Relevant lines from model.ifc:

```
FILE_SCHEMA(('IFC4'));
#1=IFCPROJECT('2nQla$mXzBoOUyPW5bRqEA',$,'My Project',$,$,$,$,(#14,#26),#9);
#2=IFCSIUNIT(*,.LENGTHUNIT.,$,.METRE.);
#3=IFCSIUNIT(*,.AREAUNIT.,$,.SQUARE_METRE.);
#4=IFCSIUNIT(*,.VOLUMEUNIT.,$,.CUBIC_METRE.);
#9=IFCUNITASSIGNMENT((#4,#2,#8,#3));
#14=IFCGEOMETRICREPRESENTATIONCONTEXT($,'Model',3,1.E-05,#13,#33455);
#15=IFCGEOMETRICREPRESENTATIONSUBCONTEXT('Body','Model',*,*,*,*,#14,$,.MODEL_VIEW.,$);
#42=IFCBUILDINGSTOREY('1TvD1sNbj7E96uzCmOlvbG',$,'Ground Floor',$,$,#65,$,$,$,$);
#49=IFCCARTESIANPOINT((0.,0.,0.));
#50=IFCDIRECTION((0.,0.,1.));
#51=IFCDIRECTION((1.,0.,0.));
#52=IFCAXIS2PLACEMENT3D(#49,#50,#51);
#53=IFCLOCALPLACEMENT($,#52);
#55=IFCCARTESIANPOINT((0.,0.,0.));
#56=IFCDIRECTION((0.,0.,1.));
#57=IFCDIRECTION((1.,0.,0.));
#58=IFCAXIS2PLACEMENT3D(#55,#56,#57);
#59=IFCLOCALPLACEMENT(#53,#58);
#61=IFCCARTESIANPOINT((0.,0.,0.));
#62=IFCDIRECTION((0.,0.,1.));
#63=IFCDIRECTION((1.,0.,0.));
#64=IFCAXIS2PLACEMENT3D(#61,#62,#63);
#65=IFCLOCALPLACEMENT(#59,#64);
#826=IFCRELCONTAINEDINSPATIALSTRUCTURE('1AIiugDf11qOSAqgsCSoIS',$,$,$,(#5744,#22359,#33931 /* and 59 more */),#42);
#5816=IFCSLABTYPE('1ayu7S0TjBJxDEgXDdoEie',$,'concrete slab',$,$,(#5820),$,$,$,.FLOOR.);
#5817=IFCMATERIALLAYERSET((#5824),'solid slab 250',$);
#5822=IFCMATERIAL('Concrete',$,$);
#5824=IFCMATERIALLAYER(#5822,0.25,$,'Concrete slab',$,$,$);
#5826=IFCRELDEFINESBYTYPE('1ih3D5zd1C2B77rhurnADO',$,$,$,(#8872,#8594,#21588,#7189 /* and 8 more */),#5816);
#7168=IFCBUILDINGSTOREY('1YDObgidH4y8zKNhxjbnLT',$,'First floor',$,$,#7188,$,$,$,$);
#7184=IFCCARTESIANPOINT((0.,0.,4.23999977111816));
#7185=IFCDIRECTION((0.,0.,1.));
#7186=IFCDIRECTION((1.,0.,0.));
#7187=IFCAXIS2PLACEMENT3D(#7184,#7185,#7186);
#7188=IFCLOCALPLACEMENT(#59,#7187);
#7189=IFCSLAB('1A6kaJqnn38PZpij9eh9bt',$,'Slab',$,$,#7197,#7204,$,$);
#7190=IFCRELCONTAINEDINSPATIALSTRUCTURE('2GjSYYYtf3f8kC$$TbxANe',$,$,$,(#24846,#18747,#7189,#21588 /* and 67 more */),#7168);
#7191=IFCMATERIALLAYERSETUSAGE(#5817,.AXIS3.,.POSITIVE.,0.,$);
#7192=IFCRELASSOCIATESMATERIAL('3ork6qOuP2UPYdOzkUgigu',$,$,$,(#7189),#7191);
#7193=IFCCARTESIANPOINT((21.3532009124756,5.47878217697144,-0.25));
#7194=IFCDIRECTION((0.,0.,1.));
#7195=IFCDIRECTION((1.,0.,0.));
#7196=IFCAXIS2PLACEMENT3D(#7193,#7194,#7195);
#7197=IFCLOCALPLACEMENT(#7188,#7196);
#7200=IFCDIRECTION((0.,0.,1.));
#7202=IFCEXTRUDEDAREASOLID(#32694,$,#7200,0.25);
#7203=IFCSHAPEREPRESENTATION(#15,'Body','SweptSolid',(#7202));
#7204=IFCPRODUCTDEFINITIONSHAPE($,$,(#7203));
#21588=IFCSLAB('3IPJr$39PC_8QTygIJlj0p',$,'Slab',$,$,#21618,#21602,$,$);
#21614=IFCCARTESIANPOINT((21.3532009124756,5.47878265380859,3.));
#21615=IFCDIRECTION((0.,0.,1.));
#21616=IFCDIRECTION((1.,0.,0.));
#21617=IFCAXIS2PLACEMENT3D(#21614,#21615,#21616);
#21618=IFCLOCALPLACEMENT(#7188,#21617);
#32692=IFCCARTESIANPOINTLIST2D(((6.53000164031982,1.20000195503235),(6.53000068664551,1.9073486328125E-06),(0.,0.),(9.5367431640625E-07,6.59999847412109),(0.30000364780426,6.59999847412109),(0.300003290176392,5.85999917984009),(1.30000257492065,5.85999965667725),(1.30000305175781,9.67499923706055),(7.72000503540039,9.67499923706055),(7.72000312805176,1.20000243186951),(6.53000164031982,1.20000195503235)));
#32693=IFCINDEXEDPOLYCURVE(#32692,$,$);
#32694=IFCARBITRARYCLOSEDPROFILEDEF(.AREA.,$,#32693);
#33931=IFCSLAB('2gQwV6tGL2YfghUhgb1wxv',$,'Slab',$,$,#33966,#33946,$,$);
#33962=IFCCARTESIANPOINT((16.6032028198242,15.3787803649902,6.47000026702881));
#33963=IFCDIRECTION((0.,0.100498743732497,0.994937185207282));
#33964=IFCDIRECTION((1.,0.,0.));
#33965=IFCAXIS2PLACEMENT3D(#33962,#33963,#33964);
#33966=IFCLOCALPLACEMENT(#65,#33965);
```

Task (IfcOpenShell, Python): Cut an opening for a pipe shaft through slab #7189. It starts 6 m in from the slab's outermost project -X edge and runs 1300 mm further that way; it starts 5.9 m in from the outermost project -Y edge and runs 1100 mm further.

```python
import numpy as np
import ifcopenshell
import ifcopenshell.api.feature
import ifcopenshell.api.geometry
import ifcopenshell.api.root
import ifcopenshell.geom
import ifcopenshell.util.placement
import ifcopenshell.util.representation
import ifcopenshell.util.shape
import ifcopenshell.util.unit

model = ifcopenshell.open("model.ifc")
unit_scale = ifcopenshell.util.unit.calculate_unit_scale(model)
settings = ifcopenshell.geom.settings()


def volume(element):
    """Net volume in cubic metres, openings subtracted."""
    shape = ifcopenshell.geom.create_shape(settings, element)
    return ifcopenshell.util.shape.get_volume(shape.geometry)


slab = model.by_guid("1A6kaJqnn38PZpij9eh9bt")
before = volume(slab)

# Extent in the slab's own axes, in metres. The edges named are its -X and -Y sides.
slab_shape = ifcopenshell.geom.create_shape(settings, slab)
vertices = ifcopenshell.util.shape.get_vertices(slab_shape.geometry)
x_min, y_min, bottom = vertices.min(axis=0)
top = vertices[:, 2].max()

opening = ifcopenshell.api.root.create_entity(model, ifc_class="IfcOpeningElement", name="Pipe shaft opening", predefined_type="OPENING")
context = ifcopenshell.util.representation.get_context(model, "Model", "Body", "MODEL_VIEW")
width, depth = 1.3, 1.1
outline = [(0.0, 0.0), (width, 0.0), (width, depth), (0.0, depth), (0.0, 0.0)]
# Overshoot both faces by 50 mm so the cut is clean.
shape = ifcopenshell.api.geometry.add_slab_representation(
    model, context=context, depth=top - bottom + 0.1, polyline=outline
)
ifcopenshell.api.geometry.assign_representation(model, product=opening, representation=shape)

matrix = ifcopenshell.util.placement.get_local_placement(slab.ObjectPlacement)
matrix[:, 3] = matrix @ np.append(np.array([x_min + 6, y_min + 5.9, bottom - 0.05]) / unit_scale, 1.0)
ifcopenshell.api.geometry.edit_object_placement(model, product=opening, matrix=matrix, is_si=False)
ifcopenshell.api.feature.add_feature(model, feature=opening, element=slab)

after = volume(slab)

print(f"slab volume {before:.3f} -> {after:.3f} m3")

model.write("model_edited.ifc")
```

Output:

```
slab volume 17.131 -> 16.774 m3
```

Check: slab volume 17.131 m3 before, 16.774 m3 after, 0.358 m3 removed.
